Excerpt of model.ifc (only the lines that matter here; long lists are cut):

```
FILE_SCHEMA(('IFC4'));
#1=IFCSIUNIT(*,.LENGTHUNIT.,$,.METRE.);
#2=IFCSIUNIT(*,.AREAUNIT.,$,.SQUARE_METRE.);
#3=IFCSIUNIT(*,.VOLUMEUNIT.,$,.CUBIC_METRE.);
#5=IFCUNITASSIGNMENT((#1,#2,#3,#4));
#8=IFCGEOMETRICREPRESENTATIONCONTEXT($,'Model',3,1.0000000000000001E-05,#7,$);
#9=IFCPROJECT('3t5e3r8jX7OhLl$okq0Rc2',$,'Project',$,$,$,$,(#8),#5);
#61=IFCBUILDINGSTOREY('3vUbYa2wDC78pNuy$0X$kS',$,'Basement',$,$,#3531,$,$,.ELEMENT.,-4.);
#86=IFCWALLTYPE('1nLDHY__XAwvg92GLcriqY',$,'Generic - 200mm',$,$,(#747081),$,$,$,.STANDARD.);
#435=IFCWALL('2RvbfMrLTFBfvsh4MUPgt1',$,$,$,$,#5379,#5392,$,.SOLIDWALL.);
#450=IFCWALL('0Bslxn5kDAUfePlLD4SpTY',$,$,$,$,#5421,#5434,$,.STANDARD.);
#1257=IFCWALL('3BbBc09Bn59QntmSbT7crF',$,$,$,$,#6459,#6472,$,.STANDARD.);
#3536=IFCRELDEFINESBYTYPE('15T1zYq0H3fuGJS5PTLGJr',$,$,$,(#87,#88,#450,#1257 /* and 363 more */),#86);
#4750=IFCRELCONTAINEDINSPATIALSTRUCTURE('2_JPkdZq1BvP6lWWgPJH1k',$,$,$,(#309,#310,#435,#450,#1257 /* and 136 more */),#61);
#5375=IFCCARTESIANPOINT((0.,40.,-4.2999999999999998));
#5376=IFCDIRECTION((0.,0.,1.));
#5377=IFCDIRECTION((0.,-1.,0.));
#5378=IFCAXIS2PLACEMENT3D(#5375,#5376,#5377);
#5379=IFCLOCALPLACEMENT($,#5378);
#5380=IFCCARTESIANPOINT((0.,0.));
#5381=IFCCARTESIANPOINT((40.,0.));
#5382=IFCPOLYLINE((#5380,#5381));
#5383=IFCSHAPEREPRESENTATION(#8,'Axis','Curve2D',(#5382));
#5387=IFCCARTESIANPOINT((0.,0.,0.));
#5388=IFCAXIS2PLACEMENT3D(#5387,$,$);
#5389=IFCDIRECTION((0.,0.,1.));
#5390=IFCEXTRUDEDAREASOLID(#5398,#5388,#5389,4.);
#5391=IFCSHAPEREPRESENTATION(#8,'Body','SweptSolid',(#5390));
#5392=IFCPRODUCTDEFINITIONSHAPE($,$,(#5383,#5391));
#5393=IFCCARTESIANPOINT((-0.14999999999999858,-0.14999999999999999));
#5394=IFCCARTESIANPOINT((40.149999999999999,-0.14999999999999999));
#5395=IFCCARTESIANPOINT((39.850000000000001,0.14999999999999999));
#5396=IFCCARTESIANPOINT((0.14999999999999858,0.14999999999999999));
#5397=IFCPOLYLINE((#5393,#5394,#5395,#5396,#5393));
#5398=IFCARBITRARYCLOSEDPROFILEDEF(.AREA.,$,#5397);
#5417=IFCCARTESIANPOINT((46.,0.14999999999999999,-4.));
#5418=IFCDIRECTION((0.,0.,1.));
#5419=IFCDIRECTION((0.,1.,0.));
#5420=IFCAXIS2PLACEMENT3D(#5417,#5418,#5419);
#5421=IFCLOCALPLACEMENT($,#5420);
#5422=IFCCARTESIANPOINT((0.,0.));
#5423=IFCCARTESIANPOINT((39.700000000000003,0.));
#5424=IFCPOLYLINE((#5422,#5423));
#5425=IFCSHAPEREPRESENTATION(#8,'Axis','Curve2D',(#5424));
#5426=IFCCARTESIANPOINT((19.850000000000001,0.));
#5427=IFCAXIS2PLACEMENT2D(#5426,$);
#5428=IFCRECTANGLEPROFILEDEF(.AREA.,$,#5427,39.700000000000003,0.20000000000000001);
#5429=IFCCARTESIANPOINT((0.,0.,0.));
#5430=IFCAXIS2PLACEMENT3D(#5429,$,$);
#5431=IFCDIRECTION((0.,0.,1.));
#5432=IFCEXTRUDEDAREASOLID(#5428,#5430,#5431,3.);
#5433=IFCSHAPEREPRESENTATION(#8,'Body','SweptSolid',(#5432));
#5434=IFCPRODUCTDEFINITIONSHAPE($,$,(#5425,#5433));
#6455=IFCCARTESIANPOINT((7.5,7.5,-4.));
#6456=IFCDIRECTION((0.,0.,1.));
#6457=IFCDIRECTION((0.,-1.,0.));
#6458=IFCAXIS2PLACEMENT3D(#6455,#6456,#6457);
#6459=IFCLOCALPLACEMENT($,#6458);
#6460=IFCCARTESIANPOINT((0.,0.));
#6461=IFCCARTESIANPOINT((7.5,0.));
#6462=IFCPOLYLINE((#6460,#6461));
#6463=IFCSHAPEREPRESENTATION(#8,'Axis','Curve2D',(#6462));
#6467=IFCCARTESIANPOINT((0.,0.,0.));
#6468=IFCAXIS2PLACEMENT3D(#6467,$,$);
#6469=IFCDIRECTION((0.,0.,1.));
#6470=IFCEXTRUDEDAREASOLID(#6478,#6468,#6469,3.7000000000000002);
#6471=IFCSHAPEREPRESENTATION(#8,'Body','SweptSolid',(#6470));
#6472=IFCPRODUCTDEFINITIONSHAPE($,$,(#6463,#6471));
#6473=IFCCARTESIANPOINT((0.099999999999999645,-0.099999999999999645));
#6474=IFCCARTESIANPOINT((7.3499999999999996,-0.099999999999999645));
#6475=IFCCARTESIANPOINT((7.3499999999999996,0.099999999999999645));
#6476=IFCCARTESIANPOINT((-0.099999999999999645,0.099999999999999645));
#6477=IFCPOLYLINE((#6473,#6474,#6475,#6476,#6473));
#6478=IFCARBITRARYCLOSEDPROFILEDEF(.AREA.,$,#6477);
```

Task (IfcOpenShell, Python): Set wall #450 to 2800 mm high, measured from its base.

```python
import ifcopenshell
import ifcopenshell.geom
import ifcopenshell.util.shape
import ifcopenshell.util.unit

model = ifcopenshell.open("model.ifc")
unit_scale = ifcopenshell.util.unit.calculate_unit_scale(model)
settings = ifcopenshell.geom.settings()


def volume(element):
    """Net volume in cubic metres, openings subtracted."""
    shape = ifcopenshell.geom.create_shape(settings, element)
    return ifcopenshell.util.shape.get_volume(shape.geometry)


wall = model.by_id(450)
before = volume(wall)

body = next(r for r in wall.Representation.Representations if r.RepresentationIdentifier == "Body")
solid = body.Items[0]
old_height = solid.Depth
solid.Depth = 2.8 / unit_scale
after = volume(wall)

print(f"height {old_height:g} -> {solid.Depth:g}, volume {before:.3f} -> {after:.3f} m3")

model.write("model_updated.ifc")
```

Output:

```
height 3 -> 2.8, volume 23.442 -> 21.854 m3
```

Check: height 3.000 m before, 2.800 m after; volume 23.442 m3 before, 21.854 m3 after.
